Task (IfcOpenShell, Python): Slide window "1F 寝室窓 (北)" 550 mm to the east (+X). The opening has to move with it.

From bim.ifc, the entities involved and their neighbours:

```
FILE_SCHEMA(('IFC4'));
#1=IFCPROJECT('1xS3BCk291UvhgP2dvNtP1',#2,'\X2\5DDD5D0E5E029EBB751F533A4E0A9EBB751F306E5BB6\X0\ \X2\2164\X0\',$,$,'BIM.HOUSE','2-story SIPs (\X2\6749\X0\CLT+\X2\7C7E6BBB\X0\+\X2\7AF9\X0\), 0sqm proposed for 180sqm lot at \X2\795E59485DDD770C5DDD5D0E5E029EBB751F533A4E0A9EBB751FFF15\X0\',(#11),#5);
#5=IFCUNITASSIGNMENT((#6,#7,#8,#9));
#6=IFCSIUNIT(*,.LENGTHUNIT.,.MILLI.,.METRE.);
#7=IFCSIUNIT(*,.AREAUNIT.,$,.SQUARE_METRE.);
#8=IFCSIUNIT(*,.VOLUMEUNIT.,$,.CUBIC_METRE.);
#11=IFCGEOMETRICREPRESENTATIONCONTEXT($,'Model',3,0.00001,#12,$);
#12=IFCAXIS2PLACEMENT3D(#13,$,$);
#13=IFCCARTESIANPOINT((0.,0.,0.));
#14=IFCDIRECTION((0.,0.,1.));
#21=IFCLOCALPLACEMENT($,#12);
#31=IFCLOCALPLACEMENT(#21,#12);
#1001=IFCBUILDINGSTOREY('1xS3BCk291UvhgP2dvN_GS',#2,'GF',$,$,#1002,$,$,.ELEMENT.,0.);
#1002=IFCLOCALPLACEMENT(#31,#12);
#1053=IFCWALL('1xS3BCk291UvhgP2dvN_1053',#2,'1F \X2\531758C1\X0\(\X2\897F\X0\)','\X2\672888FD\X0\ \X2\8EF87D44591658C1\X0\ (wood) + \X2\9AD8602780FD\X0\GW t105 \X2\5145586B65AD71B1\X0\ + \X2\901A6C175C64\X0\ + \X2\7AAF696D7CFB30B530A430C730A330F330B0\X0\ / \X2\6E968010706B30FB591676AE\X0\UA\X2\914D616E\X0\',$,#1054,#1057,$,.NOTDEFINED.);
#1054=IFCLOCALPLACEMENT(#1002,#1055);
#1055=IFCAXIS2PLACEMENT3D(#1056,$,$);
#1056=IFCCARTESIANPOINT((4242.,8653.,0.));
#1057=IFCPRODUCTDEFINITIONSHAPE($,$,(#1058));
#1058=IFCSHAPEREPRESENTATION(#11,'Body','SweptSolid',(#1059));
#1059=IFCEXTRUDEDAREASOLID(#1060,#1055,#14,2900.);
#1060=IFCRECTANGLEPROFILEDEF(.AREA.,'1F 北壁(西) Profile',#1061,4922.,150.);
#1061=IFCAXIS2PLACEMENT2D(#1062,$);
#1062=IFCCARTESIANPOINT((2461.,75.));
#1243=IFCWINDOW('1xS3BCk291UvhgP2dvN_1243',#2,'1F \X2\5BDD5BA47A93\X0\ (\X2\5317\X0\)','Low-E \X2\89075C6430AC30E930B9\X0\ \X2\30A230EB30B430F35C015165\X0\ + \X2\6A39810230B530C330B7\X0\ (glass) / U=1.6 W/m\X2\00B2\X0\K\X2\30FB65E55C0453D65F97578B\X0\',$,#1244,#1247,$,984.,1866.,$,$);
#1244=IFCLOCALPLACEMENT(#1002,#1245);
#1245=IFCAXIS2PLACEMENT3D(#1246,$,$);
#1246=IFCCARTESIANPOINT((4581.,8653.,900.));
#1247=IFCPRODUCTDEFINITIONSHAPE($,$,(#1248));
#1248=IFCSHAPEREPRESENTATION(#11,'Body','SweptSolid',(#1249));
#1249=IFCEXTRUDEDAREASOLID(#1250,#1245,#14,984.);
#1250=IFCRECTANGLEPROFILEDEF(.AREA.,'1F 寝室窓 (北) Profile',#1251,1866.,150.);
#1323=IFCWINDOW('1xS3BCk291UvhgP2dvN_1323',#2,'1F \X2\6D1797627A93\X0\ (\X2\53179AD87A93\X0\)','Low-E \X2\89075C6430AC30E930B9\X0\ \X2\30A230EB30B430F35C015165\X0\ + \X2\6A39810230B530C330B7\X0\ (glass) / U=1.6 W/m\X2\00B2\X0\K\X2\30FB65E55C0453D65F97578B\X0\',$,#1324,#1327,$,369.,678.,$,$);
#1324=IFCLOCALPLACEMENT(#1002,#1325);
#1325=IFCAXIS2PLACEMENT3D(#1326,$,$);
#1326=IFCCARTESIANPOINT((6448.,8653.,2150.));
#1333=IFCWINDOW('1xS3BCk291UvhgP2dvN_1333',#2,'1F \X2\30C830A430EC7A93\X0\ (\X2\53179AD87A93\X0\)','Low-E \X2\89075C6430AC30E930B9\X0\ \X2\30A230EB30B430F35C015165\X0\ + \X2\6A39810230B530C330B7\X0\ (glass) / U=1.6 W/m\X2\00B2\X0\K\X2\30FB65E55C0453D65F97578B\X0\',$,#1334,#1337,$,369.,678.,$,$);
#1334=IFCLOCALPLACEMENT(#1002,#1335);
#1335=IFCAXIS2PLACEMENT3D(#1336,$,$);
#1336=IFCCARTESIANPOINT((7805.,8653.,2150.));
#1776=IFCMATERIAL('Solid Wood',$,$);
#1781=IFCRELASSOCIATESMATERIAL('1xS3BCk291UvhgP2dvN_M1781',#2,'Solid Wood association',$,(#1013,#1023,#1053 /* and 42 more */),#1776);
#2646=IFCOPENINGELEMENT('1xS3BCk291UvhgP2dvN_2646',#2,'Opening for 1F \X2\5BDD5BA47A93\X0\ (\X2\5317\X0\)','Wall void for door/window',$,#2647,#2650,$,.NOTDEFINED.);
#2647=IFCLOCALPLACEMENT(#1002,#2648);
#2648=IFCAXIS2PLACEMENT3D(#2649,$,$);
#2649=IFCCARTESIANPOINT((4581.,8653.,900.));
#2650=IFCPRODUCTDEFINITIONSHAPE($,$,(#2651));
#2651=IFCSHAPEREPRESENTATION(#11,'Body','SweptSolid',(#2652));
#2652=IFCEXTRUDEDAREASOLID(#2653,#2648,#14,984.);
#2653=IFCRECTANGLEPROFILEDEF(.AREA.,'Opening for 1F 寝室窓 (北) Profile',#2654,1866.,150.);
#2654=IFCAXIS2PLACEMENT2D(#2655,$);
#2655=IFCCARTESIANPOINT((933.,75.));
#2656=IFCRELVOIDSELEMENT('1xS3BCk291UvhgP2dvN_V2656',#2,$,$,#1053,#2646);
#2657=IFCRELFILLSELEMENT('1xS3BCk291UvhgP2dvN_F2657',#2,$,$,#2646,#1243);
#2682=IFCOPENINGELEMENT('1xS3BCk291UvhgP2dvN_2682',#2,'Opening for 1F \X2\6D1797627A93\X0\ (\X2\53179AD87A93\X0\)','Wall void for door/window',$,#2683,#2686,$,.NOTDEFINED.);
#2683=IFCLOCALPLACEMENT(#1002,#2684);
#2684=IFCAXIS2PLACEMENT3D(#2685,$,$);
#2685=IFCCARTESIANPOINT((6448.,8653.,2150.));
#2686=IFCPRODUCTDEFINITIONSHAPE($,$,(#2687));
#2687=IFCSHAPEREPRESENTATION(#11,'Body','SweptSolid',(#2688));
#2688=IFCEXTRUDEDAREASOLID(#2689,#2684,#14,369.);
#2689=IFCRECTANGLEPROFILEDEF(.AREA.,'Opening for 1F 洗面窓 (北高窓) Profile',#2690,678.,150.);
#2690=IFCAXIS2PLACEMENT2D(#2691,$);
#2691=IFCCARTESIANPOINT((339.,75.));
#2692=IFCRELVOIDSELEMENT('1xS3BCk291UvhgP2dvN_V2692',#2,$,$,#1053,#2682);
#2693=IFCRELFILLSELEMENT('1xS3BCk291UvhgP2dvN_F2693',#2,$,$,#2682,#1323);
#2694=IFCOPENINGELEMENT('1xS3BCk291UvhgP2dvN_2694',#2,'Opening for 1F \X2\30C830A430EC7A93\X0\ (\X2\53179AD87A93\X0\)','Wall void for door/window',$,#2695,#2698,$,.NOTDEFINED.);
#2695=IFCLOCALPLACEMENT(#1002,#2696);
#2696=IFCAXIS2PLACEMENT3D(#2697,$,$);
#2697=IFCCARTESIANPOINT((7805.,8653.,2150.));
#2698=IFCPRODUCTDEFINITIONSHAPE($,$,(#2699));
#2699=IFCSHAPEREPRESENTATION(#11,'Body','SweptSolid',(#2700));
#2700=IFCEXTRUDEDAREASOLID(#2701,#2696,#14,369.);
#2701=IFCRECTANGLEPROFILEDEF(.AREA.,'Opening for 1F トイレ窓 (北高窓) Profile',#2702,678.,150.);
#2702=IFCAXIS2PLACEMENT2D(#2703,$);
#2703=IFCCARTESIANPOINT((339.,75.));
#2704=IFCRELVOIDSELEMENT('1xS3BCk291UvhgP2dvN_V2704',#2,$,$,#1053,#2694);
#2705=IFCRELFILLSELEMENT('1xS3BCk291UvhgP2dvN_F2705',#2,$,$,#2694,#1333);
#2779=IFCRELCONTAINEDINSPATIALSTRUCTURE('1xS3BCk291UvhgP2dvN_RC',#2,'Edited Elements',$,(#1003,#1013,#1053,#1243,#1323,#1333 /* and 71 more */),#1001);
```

```python
import ifcopenshell
import ifcopenshell.api.geometry
import ifcopenshell.util.placement

model = ifcopenshell.open("bim.ifc")

window = model.by_id(1243)
opening = window.FillsVoids[0].RelatingOpeningElement
wall = opening.VoidsElements[0].RelatingBuildingElement

wall_matrix = ifcopenshell.util.placement.get_local_placement(wall.ObjectPlacement)
shift = wall_matrix[:3, 0] * 550.0
before = ifcopenshell.util.placement.get_local_placement(window.ObjectPlacement)[:3, 3].copy()

# The window is not placed relative to its opening, so move both.
for product in (opening, window):
    matrix = ifcopenshell.util.placement.get_local_placement(product.ObjectPlacement)
    matrix[:3, 3] += shift
    ifcopenshell.api.geometry.edit_object_placement(model, product=product, matrix=matrix, is_si=False)

after = ifcopenshell.util.placement.get_local_placement(window.ObjectPlacement)[:3, 3]
print("window moved by", (after - before).round(3) + 0.0)

model.write("bim_v2.ifc")
```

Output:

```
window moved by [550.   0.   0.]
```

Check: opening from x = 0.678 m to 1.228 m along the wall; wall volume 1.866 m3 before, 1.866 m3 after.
